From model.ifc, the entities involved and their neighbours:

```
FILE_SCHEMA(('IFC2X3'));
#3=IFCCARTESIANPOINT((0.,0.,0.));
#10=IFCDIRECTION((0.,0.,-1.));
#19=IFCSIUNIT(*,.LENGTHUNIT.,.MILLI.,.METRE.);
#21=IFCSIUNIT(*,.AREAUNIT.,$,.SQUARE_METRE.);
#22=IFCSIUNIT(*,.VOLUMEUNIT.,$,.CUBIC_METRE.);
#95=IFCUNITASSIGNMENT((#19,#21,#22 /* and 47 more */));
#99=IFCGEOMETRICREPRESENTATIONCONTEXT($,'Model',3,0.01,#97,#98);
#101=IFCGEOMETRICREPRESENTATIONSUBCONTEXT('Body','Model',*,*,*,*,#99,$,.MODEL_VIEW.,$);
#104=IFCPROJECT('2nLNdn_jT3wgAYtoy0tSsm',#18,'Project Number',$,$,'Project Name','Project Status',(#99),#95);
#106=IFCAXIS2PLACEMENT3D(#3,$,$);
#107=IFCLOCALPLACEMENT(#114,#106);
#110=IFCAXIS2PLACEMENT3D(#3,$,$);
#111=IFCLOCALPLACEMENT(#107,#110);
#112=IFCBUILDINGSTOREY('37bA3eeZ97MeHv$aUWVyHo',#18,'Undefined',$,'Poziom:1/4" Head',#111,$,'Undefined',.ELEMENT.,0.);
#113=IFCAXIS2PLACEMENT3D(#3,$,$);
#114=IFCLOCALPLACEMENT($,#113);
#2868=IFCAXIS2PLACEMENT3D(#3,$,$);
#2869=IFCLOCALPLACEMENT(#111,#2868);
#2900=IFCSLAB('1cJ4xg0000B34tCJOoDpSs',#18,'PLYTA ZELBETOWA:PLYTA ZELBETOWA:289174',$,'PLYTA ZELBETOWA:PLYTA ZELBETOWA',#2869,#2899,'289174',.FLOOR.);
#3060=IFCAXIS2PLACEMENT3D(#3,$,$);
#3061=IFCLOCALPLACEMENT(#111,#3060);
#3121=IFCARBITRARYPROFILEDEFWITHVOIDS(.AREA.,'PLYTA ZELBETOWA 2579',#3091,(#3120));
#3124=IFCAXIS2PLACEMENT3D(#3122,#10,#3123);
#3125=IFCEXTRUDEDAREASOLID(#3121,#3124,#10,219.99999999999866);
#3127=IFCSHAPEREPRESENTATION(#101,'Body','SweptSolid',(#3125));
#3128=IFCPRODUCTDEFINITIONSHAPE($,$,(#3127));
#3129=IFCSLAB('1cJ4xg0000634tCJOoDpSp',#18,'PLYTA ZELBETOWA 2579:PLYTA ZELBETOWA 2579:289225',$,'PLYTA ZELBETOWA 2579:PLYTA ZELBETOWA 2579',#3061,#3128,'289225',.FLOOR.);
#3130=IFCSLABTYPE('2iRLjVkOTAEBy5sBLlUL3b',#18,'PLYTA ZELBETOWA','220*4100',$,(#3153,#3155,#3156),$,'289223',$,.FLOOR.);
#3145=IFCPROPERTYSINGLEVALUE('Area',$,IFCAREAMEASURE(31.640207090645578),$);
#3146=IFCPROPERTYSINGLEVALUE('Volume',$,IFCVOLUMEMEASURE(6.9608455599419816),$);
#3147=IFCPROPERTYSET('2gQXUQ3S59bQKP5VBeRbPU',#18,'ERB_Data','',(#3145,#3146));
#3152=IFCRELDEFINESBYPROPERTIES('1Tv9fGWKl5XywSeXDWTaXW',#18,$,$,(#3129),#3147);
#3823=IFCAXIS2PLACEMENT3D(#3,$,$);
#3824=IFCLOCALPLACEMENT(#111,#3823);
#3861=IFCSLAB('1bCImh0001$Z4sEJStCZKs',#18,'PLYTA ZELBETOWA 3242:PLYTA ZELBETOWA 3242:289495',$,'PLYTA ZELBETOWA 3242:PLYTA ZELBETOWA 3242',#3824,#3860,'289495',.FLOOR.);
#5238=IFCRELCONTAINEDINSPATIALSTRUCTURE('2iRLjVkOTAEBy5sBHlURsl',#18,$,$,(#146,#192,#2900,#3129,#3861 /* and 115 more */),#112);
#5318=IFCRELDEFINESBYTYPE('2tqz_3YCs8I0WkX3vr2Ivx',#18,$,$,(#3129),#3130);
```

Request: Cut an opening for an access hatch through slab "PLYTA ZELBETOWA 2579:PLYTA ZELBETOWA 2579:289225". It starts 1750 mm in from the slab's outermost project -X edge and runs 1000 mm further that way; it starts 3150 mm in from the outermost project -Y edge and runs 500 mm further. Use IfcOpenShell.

```python
import numpy as np
import ifcopenshell
import ifcopenshell.api.feature
import ifcopenshell.api.geometry
import ifcopenshell.api.pset
import ifcopenshell.api.root
import ifcopenshell.geom
import ifcopenshell.util.element
import ifcopenshell.util.placement
import ifcopenshell.util.representation
import ifcopenshell.util.shape
import ifcopenshell.util.unit

model = ifcopenshell.open("model.ifc")
unit_scale = ifcopenshell.util.unit.calculate_unit_scale(model)
area_scale = ifcopenshell.util.unit.calculate_unit_scale(model, "AREAUNIT")
volume_scale = ifcopenshell.util.unit.calculate_unit_scale(model, "VOLUMEUNIT")
settings = ifcopenshell.geom.settings()


def volume(element):
    """Net volume in cubic metres, openings subtracted."""
    shape = ifcopenshell.geom.create_shape(settings, element)
    return ifcopenshell.util.shape.get_volume(shape.geometry)


slab = model.by_guid("1cJ4xg0000634tCJOoDpSp")
before = volume(slab)

# Extent in the slab's own axes, in metres. The edges named are its -X and -Y sides.
slab_shape = ifcopenshell.geom.create_shape(settings, slab)
vertices = ifcopenshell.util.shape.get_vertices(slab_shape.geometry)
x_min, y_min, bottom = vertices.min(axis=0)
top = vertices[:, 2].max()

opening = ifcopenshell.api.root.create_entity(model, ifc_class="IfcOpeningElement", name="Access hatch opening")
context = ifcopenshell.util.representation.get_context(model, "Model", "Body", "MODEL_VIEW")
width, depth = 1, 0.5
outline = [(0.0, 0.0), (width, 0.0), (width, depth), (0.0, depth), (0.0, 0.0)]
# Overshoot both faces by 50 mm so the cut is clean.
shape = ifcopenshell.api.geometry.add_slab_representation(
    model, context=context, depth=top - bottom + 0.1, polyline=outline
)
ifcopenshell.api.geometry.assign_representation(model, product=opening, representation=shape)

matrix = ifcopenshell.util.placement.get_local_placement(slab.ObjectPlacement)
matrix[:, 3] = matrix @ np.append(np.array([x_min + 1.75, y_min + 3.15, bottom - 0.05]) / unit_scale, 1.0)
ifcopenshell.api.geometry.edit_object_placement(model, product=opening, matrix=matrix, is_si=False)
ifcopenshell.api.feature.add_feature(model, feature=opening, element=slab)

after = volume(slab)

# Update the slab's stored quantities.
pset = model.by_id(ifcopenshell.util.element.get_pset(slab, "ERB_Data", should_inherit=False)["id"])
ifcopenshell.api.pset.edit_pset(model, pset=pset, properties={
    "Area": model.create_entity("IfcAreaMeasure", after / (top - bottom) / area_scale),
    "Volume": model.create_entity("IfcVolumeMeasure", after / volume_scale),
})

print(f"slab volume {before:.3f} -> {after:.3f} m3")

model.write("model_edited.ifc")
```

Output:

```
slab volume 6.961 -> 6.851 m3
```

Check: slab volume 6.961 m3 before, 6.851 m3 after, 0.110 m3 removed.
